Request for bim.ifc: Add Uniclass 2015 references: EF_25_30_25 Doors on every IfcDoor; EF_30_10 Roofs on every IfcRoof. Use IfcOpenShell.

First a look at what the model holds.

```python
import ifcopenshell

model = ifcopenshell.open("bim.ifc")
print(model.schema)
print("classifications:", [c.Name for c in model.by_type("IfcClassification")])
for ifc_class in ("IfcDoor", "IfcRoof", "IfcStair", "IfcWall", "IfcWindow"):
    print(ifc_class, len(model.by_type(ifc_class)))
```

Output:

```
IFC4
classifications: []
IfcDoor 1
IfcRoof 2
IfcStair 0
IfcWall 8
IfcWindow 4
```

```python
import ifcopenshell
import ifcopenshell.api.classification

model = ifcopenshell.open("bim.ifc")

system = ifcopenshell.api.classification.add_classification(model, classification="Uniclass 2015")

codes = {
    "IfcDoor": ("EF_25_30_25", "Doors"),
    "IfcRoof": ("EF_30_10", "Roofs"),
}
for ifc_class, (code, name) in codes.items():
    products = model.by_type(ifc_class)
    ifcopenshell.api.classification.add_reference(
        model, products=products, classification=system, identification=code, name=name
    )
    print(code, len(products))

model.write("bim_rev.ifc")
```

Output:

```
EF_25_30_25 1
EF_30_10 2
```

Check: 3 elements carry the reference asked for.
